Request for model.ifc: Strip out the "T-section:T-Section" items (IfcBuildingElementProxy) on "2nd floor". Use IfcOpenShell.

First a look at what the model holds.

```python
import ifcopenshell
import ifcopenshell.util.element

model = ifcopenshell.open("model.ifc")
print(model.schema)
storey = next(s for s in model.by_type("IfcBuildingStorey") if s.Name == "2nd floor")
proxies = [e for e in ifcopenshell.util.element.get_decomposition(storey) if e.is_a("IfcBuildingElementProxy")]
seen = {}
for e in proxies:
    element_type = ifcopenshell.util.element.get_type(e)
    name = element_type.Name if element_type not in (None, e) else None
    seen[name] = seen.get(name, 0) + 1
for name, count in sorted(seen.items(), key=str):
    print(count, "x", name)
```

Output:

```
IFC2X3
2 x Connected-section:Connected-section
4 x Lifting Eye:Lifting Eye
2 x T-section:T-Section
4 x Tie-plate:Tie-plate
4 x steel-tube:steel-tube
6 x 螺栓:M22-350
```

```python
import ifcopenshell
import ifcopenshell.api.root
import ifcopenshell.util.element

model = ifcopenshell.open("model.ifc")

storey = next(s for s in model.by_type("IfcBuildingStorey") if s.Name == "2nd floor")
proxies = [e for e in ifcopenshell.util.element.get_decomposition(storey) if e.is_a("IfcBuildingElementProxy")]
targets = [e for e in proxies if (t := ifcopenshell.util.element.get_type(e)) not in (None, e) and t.Name == "T-section:T-Section"]

for e in targets:
    ifcopenshell.api.root.remove_product(model, product=e)
print(len(targets), "removed")

model.write("model-out.ifc")
```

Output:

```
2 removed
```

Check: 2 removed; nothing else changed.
